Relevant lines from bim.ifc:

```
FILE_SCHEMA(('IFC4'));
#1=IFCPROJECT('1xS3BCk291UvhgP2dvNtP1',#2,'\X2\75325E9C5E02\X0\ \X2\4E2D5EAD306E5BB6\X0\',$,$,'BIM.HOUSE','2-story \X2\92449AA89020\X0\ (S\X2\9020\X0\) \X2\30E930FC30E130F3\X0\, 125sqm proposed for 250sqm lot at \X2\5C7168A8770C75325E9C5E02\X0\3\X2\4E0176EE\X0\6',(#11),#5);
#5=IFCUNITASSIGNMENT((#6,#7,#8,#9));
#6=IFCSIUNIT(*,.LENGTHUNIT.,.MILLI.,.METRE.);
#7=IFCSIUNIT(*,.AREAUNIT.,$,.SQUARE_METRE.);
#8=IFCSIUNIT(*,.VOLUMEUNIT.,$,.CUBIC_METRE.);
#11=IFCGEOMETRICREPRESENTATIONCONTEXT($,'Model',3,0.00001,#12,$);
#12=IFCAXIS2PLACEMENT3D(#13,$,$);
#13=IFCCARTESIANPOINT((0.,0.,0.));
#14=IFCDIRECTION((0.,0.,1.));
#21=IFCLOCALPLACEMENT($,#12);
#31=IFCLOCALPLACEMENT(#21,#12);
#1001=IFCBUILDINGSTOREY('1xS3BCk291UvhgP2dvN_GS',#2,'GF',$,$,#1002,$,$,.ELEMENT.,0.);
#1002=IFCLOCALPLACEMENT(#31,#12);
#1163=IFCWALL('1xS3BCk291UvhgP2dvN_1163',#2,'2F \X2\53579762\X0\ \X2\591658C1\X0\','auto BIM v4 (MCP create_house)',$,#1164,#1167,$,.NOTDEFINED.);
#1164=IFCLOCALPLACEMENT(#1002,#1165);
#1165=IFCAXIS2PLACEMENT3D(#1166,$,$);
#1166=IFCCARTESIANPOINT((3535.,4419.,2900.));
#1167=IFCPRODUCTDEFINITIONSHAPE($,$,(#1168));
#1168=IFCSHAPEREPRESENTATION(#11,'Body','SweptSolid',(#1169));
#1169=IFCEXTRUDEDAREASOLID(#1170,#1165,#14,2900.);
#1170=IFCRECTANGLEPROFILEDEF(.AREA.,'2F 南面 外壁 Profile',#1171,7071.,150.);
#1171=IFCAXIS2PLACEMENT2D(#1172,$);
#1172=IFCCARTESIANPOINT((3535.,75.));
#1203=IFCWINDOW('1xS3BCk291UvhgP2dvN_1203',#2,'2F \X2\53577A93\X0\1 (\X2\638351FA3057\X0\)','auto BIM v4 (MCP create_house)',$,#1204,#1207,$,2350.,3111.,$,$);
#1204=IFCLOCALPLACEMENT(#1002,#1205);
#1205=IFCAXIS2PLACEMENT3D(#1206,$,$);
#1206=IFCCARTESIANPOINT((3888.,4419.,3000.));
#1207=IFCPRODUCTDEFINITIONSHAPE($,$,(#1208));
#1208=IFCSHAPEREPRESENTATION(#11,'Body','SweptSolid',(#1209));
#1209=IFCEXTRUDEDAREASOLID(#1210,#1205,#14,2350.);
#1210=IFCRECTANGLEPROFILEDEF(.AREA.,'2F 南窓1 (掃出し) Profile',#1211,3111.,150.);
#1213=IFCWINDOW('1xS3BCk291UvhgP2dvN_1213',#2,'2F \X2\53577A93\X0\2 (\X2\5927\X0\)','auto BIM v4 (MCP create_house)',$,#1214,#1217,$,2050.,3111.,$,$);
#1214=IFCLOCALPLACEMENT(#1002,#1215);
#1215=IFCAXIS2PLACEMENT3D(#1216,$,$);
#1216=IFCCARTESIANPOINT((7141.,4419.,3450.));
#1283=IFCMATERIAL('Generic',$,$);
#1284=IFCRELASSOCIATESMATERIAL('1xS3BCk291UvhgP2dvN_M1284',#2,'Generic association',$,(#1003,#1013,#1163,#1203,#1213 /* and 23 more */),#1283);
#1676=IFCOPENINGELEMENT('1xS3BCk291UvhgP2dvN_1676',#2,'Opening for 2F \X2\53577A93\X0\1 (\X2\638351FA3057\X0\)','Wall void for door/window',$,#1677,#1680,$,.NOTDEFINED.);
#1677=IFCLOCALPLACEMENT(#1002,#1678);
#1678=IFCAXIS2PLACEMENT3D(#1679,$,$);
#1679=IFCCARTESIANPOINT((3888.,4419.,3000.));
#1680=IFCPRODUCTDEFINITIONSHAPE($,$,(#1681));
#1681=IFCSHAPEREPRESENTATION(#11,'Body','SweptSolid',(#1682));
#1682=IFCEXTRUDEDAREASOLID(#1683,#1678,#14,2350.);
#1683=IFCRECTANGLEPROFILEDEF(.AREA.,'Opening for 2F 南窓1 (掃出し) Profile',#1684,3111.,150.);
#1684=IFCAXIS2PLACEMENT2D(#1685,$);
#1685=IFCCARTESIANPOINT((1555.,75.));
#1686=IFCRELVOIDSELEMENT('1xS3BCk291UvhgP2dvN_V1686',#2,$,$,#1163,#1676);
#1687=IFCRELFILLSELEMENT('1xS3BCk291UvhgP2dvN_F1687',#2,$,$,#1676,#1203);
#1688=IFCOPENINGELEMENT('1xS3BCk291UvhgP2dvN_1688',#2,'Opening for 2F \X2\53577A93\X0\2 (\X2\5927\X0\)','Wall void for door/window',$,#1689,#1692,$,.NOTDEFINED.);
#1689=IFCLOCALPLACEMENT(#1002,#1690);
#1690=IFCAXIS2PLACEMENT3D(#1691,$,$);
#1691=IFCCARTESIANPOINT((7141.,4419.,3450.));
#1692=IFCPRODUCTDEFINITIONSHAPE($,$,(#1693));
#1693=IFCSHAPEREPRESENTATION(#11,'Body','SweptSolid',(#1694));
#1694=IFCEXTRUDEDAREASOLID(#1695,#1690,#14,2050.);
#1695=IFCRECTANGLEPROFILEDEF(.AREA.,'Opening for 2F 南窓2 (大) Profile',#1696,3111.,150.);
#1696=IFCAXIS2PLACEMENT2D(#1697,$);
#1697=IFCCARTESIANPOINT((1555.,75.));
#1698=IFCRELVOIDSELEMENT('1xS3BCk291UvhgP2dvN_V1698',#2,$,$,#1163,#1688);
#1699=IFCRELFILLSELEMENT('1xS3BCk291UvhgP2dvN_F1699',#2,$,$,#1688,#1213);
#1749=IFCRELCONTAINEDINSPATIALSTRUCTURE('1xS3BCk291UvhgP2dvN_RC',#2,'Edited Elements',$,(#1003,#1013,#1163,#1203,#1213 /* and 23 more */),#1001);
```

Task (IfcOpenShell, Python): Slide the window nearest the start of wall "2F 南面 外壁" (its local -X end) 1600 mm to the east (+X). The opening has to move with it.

```python
import ifcopenshell
import ifcopenshell.api.geometry
import ifcopenshell.util.placement
import ifcopenshell.util.unit

model = ifcopenshell.open("bim.ifc")
unit_scale = ifcopenshell.util.unit.calculate_unit_scale(model)

window = model.by_guid("1xS3BCk291UvhgP2dvN_1203")
opening = window.FillsVoids[0].RelatingOpeningElement
wall = opening.VoidsElements[0].RelatingBuildingElement

wall_matrix = ifcopenshell.util.placement.get_local_placement(wall.ObjectPlacement)
shift = wall_matrix[:3, 0] * 1.6 / unit_scale
before = ifcopenshell.util.placement.get_local_placement(window.ObjectPlacement)[:3, 3].copy()

# The window is not placed relative to its opening, so move both.
for product in (opening, window):
    matrix = ifcopenshell.util.placement.get_local_placement(product.ObjectPlacement)
    matrix[:3, 3] += shift
    ifcopenshell.api.geometry.edit_object_placement(model, product=product, matrix=matrix, is_si=False)

after = ifcopenshell.util.placement.get_local_placement(window.ObjectPlacement)[:3, 3]
print("window moved by", (after - before).round(3) + 0.0)

model.write("bim-out.ifc")
```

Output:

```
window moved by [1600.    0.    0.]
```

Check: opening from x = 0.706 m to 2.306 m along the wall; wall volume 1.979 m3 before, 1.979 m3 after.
